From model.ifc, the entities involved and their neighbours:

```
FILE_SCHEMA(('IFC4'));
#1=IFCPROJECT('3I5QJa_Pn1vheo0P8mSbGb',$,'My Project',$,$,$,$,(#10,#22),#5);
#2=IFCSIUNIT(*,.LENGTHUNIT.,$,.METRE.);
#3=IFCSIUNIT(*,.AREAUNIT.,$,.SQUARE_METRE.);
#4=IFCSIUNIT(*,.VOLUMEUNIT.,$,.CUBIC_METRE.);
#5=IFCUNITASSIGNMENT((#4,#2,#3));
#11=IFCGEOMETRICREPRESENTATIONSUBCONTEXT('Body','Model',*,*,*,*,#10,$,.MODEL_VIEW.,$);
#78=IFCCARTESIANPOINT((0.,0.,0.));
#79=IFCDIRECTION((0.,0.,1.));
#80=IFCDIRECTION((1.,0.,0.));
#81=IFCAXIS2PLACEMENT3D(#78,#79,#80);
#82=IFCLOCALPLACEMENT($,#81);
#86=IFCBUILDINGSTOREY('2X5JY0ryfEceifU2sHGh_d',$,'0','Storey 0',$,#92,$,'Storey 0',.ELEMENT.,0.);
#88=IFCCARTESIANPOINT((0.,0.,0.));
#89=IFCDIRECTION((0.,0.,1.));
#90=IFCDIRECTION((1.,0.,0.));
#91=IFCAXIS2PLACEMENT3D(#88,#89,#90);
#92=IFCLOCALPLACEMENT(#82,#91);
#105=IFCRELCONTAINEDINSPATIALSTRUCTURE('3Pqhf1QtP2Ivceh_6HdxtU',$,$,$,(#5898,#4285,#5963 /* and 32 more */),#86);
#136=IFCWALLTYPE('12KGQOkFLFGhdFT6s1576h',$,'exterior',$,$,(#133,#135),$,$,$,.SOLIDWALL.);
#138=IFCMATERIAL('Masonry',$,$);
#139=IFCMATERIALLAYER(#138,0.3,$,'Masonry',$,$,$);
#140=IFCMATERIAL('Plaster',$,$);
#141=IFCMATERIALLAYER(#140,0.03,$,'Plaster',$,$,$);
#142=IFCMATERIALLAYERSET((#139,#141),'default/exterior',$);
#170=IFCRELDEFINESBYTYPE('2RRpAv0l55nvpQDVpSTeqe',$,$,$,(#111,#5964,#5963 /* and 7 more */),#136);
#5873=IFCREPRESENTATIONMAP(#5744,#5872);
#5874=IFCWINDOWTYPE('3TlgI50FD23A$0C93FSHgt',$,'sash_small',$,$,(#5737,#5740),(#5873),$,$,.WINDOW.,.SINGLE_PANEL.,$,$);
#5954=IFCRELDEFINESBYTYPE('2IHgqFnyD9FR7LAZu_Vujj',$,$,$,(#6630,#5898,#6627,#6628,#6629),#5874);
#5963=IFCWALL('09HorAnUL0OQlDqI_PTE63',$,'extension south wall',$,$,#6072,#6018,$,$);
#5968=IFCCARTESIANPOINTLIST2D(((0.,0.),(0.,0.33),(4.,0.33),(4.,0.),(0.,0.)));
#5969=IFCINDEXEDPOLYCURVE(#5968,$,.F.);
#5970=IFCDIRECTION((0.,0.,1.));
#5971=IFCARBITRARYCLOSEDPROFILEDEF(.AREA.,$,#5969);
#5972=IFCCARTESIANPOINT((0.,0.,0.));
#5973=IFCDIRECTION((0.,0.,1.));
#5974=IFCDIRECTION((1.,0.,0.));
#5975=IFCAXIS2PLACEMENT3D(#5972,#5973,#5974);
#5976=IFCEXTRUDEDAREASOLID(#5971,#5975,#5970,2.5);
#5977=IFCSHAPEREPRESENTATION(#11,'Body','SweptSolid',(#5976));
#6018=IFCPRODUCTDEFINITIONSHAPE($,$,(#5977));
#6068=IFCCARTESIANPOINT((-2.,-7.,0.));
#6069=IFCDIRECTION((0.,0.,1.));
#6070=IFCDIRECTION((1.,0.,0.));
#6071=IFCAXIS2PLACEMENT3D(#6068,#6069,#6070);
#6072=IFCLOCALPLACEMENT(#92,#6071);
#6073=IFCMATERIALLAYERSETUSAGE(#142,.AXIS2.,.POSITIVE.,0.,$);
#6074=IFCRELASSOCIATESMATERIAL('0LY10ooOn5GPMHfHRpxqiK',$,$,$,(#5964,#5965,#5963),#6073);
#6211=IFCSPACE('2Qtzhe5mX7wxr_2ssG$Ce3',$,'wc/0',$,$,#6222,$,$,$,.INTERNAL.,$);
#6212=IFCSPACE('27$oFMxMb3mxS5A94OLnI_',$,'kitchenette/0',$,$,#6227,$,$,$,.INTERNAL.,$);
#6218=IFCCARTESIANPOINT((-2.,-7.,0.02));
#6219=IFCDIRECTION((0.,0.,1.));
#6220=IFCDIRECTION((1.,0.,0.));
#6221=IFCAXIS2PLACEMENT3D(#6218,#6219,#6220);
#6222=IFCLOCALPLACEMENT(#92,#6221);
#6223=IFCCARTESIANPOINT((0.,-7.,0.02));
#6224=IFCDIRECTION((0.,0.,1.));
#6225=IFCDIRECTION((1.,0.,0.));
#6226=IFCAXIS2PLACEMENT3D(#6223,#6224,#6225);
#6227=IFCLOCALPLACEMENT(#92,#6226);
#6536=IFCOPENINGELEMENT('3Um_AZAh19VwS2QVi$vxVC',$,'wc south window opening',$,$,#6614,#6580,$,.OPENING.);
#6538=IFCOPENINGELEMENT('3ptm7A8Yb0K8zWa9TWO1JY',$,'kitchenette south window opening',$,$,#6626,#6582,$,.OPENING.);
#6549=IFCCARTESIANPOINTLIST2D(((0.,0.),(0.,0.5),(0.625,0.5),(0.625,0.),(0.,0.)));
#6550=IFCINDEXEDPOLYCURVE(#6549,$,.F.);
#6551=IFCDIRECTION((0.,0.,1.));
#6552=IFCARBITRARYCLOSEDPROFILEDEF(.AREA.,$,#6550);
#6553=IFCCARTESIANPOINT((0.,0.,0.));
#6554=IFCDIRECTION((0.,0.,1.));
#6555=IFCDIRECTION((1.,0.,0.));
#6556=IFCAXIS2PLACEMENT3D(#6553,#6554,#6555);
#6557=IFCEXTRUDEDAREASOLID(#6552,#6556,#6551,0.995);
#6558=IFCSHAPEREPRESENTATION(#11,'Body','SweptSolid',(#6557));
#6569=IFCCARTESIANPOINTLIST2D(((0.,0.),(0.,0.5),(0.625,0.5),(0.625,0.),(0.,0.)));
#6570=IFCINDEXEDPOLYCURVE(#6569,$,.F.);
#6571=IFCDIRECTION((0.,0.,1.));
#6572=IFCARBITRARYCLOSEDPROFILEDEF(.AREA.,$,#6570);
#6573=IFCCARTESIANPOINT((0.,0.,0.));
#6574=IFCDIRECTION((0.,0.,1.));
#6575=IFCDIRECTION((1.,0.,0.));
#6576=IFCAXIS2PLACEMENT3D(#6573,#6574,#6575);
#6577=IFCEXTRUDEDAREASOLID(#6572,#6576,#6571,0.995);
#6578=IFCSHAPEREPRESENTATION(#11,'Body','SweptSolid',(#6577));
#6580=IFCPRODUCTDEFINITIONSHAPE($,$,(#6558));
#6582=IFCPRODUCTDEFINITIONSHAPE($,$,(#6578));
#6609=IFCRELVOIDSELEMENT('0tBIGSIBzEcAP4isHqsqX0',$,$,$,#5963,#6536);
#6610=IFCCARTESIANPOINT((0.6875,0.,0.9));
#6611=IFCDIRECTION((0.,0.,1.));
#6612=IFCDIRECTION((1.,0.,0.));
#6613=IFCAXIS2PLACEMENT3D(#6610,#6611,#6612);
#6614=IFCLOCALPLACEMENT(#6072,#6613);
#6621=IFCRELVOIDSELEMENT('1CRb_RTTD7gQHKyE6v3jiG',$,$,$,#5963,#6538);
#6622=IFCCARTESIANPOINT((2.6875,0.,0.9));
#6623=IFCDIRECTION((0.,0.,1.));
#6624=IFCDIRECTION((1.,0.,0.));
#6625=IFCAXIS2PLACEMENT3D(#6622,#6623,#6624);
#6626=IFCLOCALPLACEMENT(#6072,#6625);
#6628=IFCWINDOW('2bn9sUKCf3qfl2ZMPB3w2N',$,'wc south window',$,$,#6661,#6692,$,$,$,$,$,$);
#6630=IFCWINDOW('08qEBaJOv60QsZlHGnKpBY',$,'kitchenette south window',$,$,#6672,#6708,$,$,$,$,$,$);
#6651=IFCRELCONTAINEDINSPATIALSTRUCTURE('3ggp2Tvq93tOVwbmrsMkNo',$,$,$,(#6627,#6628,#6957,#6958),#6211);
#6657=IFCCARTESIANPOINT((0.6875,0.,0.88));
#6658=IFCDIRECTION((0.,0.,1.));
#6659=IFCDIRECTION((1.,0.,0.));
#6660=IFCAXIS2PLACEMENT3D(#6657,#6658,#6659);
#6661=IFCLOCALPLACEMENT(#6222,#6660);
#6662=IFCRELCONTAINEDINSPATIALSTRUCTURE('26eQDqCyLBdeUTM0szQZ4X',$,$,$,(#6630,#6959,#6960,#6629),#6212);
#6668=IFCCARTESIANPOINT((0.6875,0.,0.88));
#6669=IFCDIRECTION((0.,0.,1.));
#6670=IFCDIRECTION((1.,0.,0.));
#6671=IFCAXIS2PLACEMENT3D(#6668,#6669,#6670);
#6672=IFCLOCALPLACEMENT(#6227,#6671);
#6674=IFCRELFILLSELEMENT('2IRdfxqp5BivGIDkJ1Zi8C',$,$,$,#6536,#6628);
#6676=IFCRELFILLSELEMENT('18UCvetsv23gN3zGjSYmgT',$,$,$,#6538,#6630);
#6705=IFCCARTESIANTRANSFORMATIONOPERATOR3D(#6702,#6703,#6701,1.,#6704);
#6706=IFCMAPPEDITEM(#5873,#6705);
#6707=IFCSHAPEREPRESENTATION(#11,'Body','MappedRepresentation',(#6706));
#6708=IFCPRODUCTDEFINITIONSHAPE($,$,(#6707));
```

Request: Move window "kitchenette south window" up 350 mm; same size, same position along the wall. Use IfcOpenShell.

```python
import numpy as np
import ifcopenshell
import ifcopenshell.api.geometry
import ifcopenshell.util.placement
import ifcopenshell.util.unit

model = ifcopenshell.open("model.ifc")
unit_scale = ifcopenshell.util.unit.calculate_unit_scale(model)

window = model.by_id(6630)
opening = window.FillsVoids[0].RelatingOpeningElement
dz = 0.35 / unit_scale

shift = np.array([0.0, 0.0, dz])
# The window is not placed relative to its opening, so move both.
for product in (opening, window):
    matrix = ifcopenshell.util.placement.get_local_placement(product.ObjectPlacement)
    matrix[:3, 3] += shift
    ifcopenshell.api.geometry.edit_object_placement(model, product=product, matrix=matrix, is_si=False)

print(f"moved by {dz * unit_scale:+.3f} m")

model.write("model_v2.ifc")
```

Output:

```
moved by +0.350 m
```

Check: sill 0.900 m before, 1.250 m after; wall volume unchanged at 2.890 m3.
